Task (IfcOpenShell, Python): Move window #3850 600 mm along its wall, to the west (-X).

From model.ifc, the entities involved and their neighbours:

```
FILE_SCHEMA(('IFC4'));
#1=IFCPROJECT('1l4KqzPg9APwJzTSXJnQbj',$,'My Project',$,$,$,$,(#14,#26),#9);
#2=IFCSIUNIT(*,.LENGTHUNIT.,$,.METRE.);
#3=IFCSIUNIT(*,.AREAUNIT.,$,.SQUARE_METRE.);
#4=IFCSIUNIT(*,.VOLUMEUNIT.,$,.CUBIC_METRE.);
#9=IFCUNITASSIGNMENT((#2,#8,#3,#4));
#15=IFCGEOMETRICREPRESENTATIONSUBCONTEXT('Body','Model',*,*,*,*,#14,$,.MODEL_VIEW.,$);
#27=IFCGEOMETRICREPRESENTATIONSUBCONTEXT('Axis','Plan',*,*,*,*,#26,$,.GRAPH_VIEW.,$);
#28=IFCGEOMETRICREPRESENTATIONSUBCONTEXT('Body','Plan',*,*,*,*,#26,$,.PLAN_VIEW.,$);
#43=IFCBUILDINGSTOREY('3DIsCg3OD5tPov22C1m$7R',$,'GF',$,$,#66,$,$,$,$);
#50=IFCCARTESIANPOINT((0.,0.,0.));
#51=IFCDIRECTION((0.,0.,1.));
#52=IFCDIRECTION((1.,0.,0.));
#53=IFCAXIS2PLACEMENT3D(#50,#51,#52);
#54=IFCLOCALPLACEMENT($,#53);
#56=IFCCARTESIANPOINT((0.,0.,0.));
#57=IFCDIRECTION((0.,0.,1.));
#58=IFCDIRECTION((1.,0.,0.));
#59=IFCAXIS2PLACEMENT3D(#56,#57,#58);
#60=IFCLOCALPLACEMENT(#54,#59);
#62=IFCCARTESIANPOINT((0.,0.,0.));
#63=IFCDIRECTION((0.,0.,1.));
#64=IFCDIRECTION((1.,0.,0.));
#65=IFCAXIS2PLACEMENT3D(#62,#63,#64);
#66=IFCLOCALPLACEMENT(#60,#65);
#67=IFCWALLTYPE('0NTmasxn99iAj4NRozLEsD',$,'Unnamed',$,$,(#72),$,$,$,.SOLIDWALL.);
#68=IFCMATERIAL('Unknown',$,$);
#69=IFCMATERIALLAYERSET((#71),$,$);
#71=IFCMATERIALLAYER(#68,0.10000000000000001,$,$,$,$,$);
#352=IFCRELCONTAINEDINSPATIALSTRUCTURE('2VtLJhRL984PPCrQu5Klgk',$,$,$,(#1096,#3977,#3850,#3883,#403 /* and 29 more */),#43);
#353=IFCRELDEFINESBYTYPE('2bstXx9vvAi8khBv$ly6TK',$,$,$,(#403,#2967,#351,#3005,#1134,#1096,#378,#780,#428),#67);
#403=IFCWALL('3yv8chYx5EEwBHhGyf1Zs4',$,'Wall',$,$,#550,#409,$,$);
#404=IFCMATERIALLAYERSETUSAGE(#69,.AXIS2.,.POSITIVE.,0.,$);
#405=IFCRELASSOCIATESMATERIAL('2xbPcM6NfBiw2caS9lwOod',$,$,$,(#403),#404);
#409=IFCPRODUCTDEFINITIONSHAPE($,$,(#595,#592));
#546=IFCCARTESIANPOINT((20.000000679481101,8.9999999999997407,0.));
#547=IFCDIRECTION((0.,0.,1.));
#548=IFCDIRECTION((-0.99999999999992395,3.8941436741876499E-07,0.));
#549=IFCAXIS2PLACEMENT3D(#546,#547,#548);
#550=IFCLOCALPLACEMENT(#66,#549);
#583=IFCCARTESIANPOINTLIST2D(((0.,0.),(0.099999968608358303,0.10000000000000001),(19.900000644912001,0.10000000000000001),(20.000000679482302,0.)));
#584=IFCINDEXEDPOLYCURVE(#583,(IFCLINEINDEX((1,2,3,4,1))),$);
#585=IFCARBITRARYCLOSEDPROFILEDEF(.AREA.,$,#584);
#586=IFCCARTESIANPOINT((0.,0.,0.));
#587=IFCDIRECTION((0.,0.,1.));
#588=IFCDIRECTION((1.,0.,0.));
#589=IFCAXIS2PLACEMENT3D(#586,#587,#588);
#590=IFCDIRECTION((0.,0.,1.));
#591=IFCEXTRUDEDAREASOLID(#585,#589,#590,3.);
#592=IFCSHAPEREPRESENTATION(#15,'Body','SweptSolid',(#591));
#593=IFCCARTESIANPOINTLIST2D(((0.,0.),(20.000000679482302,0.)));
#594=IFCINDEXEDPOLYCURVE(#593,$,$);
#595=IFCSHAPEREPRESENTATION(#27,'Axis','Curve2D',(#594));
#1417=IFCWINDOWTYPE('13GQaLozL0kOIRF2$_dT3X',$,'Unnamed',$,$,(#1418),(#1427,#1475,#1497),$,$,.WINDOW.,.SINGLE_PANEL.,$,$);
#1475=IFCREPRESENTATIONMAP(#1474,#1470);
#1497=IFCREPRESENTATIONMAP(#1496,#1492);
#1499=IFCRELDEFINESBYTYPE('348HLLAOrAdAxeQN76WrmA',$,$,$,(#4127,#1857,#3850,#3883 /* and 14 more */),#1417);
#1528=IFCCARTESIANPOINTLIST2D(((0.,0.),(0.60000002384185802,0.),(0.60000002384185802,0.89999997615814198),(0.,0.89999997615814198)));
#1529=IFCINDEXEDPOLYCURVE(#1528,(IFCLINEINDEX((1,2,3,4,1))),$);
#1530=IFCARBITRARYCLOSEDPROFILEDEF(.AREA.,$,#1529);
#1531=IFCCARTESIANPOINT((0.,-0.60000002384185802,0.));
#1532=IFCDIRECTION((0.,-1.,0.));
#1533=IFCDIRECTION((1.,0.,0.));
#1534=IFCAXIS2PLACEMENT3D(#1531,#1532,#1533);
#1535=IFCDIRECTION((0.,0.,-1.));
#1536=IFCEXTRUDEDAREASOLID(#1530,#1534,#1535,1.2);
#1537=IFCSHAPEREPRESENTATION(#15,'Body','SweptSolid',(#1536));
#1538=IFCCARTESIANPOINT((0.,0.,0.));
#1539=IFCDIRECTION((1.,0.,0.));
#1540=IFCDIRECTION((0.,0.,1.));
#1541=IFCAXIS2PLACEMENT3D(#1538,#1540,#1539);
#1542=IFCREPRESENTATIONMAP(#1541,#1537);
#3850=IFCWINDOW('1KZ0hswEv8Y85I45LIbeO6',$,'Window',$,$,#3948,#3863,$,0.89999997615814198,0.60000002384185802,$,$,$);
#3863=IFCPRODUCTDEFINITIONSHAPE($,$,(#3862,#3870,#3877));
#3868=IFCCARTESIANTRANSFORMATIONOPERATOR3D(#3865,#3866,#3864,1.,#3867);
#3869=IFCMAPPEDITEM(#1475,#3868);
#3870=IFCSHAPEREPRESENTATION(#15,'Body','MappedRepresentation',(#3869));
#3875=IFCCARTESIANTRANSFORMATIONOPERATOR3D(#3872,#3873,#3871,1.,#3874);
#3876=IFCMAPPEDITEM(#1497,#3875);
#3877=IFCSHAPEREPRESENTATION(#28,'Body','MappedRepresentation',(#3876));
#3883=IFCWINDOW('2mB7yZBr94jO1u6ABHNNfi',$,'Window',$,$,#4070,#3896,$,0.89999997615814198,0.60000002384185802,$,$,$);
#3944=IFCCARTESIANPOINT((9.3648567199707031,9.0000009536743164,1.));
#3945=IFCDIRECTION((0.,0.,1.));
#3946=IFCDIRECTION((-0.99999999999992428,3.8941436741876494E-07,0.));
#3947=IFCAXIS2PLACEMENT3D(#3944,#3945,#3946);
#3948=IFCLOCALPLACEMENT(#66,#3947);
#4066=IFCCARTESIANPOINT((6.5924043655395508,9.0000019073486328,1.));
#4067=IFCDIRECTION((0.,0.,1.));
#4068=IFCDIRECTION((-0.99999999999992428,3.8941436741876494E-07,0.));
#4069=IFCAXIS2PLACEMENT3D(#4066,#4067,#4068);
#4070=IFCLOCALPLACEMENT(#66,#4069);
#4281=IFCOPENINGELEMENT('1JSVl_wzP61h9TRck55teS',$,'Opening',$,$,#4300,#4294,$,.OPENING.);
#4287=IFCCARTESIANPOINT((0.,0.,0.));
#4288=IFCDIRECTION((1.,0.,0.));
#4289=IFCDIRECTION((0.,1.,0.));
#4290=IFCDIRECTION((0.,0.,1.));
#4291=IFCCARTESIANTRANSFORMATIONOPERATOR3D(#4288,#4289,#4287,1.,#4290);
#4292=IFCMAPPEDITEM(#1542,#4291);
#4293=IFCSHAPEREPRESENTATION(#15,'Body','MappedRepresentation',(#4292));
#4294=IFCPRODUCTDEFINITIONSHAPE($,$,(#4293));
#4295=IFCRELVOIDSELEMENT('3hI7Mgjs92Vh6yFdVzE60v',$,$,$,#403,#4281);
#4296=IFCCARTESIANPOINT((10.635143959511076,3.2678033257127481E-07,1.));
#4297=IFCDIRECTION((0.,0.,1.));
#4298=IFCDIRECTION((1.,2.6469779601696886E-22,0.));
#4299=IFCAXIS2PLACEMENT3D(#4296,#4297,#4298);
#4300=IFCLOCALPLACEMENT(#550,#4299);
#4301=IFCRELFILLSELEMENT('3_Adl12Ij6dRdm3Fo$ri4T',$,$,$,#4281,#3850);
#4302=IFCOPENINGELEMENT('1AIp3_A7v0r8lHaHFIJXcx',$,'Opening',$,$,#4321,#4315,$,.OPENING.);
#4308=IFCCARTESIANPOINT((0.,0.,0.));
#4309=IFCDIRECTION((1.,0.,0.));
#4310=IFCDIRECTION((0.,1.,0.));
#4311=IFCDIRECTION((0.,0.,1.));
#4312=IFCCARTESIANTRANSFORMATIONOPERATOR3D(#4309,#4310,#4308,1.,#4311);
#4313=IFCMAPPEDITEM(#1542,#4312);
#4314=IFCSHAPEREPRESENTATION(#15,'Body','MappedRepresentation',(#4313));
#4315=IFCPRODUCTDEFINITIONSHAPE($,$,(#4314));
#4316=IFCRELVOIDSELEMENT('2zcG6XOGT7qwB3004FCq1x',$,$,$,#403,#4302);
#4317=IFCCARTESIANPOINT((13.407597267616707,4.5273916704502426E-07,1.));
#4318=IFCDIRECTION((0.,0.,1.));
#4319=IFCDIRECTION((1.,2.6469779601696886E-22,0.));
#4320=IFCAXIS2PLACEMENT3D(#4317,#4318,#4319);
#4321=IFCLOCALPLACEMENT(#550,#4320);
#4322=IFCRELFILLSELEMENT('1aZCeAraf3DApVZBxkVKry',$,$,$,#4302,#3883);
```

```python
import ifcopenshell
import ifcopenshell.api.geometry
import ifcopenshell.util.placement
import ifcopenshell.util.unit

model = ifcopenshell.open("model.ifc")
unit_scale = ifcopenshell.util.unit.calculate_unit_scale(model)

window = model.by_guid("1KZ0hswEv8Y85I45LIbeO6")
opening = window.FillsVoids[0].RelatingOpeningElement
wall = opening.VoidsElements[0].RelatingBuildingElement

wall_matrix = ifcopenshell.util.placement.get_local_placement(wall.ObjectPlacement)
shift = wall_matrix[:3, 0] * 0.6 / unit_scale
before = ifcopenshell.util.placement.get_local_placement(window.ObjectPlacement)[:3, 3].copy()

# The window is not placed relative to its opening, so move both.
for product in (opening, window):
    matrix = ifcopenshell.util.placement.get_local_placement(product.ObjectPlacement)
    matrix[:3, 3] += shift
    ifcopenshell.api.geometry.edit_object_placement(model, product=product, matrix=matrix, is_si=False)

after = ifcopenshell.util.placement.get_local_placement(window.ObjectPlacement)[:3, 3]
print("window moved by", (after - before).round(3) + 0.0)

model.write("model_v2.ifc")
```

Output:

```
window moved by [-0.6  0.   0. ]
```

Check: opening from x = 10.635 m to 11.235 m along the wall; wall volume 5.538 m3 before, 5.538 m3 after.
